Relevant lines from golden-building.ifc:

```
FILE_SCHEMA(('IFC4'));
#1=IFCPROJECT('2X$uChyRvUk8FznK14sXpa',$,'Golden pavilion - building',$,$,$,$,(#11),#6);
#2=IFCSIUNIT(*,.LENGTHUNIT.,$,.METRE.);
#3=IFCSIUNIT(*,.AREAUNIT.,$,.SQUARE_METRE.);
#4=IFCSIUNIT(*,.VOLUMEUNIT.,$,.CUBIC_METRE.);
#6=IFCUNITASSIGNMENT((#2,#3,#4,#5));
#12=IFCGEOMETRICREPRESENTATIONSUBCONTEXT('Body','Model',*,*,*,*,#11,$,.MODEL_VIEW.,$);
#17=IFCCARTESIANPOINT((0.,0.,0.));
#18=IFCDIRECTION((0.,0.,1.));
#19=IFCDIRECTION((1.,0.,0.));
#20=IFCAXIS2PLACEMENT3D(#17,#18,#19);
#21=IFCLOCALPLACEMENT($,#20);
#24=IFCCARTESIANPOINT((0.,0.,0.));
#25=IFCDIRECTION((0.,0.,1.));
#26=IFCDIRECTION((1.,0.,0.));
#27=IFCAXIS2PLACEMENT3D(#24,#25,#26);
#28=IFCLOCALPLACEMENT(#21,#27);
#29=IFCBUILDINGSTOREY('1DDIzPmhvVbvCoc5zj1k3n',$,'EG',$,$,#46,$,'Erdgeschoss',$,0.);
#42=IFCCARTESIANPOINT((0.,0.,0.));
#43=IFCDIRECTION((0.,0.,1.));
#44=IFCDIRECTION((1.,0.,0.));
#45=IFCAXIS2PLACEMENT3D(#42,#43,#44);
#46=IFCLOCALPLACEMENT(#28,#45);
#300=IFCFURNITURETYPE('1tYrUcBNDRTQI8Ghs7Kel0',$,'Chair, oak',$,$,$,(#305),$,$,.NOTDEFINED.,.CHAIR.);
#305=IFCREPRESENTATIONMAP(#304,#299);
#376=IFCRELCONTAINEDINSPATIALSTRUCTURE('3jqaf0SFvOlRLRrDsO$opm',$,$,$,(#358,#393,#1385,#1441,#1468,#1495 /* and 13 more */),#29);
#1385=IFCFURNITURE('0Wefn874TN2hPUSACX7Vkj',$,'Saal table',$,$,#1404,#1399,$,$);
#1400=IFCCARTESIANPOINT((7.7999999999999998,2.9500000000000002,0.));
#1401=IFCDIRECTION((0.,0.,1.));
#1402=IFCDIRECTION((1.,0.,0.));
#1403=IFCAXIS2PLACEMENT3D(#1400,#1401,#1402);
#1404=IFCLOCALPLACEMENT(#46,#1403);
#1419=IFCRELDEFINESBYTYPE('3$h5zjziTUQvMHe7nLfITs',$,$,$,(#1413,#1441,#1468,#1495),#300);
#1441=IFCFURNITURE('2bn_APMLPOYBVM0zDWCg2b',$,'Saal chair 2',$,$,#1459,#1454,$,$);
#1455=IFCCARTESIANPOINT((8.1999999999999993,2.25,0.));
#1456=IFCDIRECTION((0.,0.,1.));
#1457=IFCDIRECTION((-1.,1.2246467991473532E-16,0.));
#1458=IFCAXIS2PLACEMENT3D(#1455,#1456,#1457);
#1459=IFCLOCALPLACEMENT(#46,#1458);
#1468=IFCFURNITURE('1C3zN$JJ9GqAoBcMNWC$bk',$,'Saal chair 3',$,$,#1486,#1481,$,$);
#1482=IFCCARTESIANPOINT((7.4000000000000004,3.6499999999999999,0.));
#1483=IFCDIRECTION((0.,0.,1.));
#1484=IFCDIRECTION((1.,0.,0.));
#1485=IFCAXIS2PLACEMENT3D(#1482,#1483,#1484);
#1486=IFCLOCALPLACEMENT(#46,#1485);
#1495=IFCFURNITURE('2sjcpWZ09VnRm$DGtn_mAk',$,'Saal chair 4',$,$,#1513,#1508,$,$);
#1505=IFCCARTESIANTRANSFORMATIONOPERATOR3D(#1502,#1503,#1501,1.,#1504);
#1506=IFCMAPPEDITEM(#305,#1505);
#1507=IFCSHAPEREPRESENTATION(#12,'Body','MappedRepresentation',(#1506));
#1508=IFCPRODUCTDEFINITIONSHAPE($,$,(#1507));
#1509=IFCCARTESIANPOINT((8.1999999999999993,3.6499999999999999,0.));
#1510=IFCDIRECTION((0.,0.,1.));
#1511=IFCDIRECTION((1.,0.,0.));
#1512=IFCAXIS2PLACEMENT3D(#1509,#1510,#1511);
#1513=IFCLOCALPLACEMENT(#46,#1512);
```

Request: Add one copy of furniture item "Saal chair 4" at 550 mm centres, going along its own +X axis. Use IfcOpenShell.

```python
import ifcopenshell
import ifcopenshell.api.geometry
import ifcopenshell.api.root
import ifcopenshell.util.element
import ifcopenshell.util.placement
import ifcopenshell.util.unit

model = ifcopenshell.open("golden-building.ifc")
unit_scale = ifcopenshell.util.unit.calculate_unit_scale(model)

source = model.by_guid("2sjcpWZ09VnRm$DGtn_mAk")
base = ifcopenshell.util.placement.get_local_placement(source.ObjectPlacement)
step = base[:3, 0] * 0.55 / unit_scale

for i in range(1, 2):
    copy = ifcopenshell.api.root.copy_class(model, product=source)
    copy.Representation = ifcopenshell.util.element.copy_deep(
        model, source.Representation, exclude=["IfcGeometricRepresentationContext", "IfcRepresentationMap"]
    )
    matrix = base.copy()
    matrix[:3, 3] += i * step
    print("added at", matrix[:3, 3].round(3) + 0.0)
    ifcopenshell.api.geometry.edit_object_placement(model, product=copy, matrix=matrix, is_si=False)

model.write("golden-building_updated.ifc")
```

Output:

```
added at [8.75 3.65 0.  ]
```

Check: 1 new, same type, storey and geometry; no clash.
